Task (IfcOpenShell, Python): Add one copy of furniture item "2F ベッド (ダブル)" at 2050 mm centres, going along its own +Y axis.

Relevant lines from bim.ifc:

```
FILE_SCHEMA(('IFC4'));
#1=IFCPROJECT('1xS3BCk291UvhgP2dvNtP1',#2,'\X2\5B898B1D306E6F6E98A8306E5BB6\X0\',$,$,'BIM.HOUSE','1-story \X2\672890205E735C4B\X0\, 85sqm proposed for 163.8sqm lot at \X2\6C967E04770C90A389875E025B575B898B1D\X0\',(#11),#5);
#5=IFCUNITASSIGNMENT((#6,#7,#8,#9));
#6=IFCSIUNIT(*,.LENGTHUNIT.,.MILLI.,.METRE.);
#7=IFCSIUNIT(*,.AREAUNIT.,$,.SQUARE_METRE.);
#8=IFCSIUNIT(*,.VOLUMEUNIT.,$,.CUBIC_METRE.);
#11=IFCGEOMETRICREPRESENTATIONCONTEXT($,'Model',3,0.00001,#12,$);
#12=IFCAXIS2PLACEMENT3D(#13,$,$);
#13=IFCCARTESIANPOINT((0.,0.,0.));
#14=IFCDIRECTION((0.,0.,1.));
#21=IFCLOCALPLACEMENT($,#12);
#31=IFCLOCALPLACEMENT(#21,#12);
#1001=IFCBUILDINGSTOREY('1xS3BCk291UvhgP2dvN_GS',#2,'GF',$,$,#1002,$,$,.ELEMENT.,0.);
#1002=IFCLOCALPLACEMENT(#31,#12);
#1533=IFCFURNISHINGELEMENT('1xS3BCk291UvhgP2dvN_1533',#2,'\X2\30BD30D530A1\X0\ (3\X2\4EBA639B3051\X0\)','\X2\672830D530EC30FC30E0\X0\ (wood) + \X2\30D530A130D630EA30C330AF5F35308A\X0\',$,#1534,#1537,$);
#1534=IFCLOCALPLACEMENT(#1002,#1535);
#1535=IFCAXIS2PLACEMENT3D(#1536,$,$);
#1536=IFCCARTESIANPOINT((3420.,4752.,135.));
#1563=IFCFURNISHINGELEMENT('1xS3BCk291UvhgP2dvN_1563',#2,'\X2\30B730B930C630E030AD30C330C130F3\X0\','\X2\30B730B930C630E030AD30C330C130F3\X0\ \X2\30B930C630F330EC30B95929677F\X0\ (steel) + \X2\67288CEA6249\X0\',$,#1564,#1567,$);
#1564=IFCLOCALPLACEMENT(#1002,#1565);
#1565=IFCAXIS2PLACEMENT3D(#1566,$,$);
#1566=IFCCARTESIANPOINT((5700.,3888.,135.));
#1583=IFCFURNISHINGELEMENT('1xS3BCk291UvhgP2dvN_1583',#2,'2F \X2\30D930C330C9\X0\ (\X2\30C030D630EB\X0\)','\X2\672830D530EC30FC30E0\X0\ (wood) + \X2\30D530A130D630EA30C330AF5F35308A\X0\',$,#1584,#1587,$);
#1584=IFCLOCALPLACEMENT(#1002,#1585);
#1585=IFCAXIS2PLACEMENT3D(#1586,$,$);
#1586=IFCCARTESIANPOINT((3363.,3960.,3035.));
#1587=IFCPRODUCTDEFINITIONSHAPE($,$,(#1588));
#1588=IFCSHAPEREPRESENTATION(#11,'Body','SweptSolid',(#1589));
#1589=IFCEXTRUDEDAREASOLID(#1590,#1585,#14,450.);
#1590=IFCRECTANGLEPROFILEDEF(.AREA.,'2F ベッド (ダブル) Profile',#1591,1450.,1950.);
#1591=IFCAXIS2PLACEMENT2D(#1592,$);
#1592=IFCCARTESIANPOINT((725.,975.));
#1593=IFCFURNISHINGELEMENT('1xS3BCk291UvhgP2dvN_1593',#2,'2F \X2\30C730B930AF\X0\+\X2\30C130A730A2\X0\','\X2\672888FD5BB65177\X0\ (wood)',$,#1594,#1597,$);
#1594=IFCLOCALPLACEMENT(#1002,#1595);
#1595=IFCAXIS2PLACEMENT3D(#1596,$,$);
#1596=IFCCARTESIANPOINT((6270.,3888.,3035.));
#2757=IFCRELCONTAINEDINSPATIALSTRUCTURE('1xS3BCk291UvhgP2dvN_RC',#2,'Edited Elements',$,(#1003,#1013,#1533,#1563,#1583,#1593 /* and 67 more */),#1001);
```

```python
import ifcopenshell
import ifcopenshell.api.geometry
import ifcopenshell.api.root
import ifcopenshell.util.element
import ifcopenshell.util.placement
import ifcopenshell.util.unit

model = ifcopenshell.open("bim.ifc")
unit_scale = ifcopenshell.util.unit.calculate_unit_scale(model)


def reuse_history(source, copy):
    """copy_class also copies each property set's owner history, people and application; keep the originals."""
    for rel in copy.IsDefinedBy:
        if rel.is_a("IfcRelDefinesByProperties") and (history := rel.RelatingPropertyDefinition.OwnerHistory):
            rel.RelatingPropertyDefinition.OwnerHistory = source.OwnerHistory
            ifcopenshell.util.element.remove_deep2(model, history)


source = model.by_guid("1xS3BCk291UvhgP2dvN_1583")
base = ifcopenshell.util.placement.get_local_placement(source.ObjectPlacement)
step = base[:3, 1] * 2.05 / unit_scale

for i in range(1, 2):
    copy = ifcopenshell.api.root.copy_class(model, product=source)
    copy.Representation = ifcopenshell.util.element.copy_deep(
        model, source.Representation, exclude=["IfcGeometricRepresentationContext", "IfcRepresentationMap"]
    )
    reuse_history(source, copy)
    matrix = base.copy()
    matrix[:3, 3] += i * step
    print("added at", matrix[:3, 3].round(3) + 0.0)
    ifcopenshell.api.geometry.edit_object_placement(model, product=copy, matrix=matrix, is_si=False)

model.write("bim_edited.ifc")
```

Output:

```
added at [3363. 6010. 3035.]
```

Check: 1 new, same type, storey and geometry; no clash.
